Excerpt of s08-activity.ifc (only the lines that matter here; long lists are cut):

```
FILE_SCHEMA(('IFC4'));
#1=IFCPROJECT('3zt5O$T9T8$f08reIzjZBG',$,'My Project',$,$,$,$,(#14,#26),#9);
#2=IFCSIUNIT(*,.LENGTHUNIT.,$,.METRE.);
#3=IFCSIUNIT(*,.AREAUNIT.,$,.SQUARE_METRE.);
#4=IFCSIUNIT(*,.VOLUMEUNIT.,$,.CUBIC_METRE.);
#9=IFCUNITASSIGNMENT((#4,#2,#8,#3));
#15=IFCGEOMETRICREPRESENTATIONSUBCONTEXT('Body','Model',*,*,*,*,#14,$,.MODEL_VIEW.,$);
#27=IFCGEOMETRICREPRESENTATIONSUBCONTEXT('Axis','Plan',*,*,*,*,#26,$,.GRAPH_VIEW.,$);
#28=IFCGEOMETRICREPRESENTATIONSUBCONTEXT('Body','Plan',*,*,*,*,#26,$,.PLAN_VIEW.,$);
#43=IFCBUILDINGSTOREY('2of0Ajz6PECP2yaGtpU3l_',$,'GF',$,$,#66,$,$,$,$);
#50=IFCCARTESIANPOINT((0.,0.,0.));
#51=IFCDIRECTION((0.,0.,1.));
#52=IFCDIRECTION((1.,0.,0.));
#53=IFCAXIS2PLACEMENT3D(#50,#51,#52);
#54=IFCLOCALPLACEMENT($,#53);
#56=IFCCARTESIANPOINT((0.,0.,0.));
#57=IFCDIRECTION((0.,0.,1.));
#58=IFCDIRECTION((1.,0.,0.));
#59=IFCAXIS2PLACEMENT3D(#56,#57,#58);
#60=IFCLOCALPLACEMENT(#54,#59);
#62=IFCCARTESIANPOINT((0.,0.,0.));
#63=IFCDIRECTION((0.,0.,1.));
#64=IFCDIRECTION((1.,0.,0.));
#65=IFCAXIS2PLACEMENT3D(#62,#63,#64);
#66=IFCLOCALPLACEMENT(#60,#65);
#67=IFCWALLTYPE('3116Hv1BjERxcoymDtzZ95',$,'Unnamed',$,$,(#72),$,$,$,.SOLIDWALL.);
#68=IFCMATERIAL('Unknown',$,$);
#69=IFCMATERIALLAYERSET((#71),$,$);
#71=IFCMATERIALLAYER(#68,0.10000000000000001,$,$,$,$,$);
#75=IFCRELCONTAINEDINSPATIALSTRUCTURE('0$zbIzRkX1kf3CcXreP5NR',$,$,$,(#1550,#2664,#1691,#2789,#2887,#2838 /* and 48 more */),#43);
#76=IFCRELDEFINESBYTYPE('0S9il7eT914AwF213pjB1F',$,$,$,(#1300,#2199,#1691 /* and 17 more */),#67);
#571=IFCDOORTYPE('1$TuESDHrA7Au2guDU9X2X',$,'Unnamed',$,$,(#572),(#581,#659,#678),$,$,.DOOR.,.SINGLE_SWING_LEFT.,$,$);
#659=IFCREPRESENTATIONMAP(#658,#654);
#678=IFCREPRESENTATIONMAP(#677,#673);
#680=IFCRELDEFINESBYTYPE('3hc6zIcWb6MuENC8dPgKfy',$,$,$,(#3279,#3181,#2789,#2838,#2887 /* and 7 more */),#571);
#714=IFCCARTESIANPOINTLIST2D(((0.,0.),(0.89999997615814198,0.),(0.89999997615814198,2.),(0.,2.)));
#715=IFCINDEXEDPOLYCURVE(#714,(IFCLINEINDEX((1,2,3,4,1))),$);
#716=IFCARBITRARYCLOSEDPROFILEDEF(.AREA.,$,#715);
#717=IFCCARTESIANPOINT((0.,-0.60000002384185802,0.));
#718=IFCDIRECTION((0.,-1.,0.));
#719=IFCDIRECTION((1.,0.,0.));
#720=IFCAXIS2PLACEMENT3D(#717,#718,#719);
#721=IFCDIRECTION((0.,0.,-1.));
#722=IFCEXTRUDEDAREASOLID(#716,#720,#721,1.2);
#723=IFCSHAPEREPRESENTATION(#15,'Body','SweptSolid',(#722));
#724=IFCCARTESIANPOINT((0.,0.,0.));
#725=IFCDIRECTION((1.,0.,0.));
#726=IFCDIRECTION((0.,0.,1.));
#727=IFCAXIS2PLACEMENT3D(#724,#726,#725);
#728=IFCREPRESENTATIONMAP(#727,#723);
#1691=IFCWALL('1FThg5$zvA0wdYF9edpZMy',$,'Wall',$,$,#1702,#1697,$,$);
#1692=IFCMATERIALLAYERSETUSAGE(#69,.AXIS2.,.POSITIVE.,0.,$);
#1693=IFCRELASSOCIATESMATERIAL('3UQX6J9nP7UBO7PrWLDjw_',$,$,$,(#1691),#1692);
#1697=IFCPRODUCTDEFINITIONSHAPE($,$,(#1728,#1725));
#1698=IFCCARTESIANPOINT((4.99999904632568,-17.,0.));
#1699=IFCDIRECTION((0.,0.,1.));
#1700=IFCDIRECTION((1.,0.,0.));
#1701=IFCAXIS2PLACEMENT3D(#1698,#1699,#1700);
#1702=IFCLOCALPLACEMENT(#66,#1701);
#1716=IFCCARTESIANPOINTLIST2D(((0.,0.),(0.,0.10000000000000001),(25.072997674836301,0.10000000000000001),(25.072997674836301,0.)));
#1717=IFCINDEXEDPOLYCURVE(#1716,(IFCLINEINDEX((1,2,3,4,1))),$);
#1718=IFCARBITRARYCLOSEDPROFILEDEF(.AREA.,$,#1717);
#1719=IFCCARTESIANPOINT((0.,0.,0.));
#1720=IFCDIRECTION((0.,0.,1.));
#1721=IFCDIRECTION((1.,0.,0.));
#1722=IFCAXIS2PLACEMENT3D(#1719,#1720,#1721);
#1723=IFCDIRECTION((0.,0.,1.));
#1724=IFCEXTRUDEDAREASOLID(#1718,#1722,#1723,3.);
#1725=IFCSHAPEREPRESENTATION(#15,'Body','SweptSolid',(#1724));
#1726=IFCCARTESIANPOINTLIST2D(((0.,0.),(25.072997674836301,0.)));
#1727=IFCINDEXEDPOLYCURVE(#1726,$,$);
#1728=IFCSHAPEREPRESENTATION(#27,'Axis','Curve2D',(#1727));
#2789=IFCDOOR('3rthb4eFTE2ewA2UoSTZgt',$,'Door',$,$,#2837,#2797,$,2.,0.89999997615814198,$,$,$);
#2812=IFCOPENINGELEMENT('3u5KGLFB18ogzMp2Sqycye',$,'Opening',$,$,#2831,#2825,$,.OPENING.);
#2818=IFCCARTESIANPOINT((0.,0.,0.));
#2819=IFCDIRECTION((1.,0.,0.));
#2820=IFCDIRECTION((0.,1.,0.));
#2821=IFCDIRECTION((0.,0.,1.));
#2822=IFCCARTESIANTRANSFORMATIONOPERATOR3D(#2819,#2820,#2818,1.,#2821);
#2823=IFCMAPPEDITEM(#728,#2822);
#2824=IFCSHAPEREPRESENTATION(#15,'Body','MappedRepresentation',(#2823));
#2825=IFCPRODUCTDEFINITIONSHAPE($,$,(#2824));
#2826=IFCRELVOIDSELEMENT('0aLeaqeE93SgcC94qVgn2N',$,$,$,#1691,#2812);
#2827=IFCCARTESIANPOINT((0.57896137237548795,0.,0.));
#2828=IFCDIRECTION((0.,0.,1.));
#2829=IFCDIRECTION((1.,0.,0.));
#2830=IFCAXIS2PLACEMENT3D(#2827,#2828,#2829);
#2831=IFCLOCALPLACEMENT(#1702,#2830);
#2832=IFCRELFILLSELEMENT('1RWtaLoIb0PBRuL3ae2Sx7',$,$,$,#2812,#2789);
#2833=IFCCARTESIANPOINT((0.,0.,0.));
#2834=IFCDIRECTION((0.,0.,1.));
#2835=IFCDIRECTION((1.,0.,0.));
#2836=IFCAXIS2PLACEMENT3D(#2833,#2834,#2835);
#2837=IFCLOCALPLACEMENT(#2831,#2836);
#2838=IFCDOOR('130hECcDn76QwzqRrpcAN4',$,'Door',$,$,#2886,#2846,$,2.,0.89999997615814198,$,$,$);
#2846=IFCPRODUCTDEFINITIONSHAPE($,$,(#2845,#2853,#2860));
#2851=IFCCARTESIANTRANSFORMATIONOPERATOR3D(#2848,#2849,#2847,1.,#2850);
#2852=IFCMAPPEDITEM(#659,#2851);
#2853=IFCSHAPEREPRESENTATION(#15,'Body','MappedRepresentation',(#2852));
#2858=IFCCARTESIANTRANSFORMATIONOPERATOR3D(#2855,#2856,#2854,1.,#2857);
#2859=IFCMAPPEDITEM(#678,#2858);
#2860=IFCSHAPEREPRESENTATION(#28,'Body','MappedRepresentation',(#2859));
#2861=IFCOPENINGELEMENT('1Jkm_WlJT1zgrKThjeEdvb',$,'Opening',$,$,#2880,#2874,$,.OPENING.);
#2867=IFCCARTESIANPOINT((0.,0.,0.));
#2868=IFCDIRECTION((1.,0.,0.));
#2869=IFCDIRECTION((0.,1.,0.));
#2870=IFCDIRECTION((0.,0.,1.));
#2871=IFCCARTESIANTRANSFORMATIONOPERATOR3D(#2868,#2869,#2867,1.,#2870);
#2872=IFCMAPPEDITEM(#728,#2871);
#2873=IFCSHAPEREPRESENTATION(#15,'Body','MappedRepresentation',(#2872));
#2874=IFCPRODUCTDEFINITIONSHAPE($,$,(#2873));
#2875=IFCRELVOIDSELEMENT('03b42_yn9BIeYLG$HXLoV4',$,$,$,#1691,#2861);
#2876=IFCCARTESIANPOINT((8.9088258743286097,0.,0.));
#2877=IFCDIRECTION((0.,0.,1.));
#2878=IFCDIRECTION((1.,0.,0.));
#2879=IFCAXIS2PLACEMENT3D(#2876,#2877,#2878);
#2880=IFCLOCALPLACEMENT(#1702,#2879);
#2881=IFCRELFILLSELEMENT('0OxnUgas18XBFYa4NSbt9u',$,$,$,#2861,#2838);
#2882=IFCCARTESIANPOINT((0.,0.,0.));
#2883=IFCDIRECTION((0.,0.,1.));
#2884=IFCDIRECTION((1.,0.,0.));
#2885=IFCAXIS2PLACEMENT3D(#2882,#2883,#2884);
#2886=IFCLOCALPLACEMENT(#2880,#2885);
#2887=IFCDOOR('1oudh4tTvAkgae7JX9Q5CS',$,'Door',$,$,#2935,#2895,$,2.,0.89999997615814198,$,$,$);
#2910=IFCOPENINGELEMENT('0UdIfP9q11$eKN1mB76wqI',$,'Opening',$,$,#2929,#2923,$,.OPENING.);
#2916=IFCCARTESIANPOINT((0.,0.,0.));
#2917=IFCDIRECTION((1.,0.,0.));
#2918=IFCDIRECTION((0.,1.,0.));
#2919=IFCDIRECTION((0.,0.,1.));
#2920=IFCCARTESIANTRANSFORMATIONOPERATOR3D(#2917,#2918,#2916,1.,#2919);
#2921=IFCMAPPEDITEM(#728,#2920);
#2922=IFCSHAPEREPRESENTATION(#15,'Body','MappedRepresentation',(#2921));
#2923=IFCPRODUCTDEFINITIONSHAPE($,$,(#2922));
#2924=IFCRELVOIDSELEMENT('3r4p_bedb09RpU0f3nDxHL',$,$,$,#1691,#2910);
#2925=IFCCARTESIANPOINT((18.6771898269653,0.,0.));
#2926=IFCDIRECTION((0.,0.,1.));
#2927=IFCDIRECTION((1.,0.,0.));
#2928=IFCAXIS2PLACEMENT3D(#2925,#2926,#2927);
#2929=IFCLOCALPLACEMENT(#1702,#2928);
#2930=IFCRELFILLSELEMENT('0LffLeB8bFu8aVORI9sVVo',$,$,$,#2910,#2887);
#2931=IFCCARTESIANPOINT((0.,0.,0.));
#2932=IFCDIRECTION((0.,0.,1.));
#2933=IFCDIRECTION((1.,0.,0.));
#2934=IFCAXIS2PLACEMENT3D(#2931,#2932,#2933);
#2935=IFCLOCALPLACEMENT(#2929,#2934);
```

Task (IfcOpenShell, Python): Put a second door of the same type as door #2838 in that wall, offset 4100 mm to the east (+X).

```python
import ifcopenshell
import ifcopenshell.api.feature
import ifcopenshell.api.geometry
import ifcopenshell.api.root
import ifcopenshell.geom
import ifcopenshell.util.element
import ifcopenshell.util.placement
import ifcopenshell.util.shape

model = ifcopenshell.open("s08-activity.ifc")
settings = ifcopenshell.geom.settings()


def volume(element):
    """Net volume in cubic metres, openings subtracted."""
    shape = ifcopenshell.geom.create_shape(settings, element)
    return ifcopenshell.util.shape.get_volume(shape.geometry)


door = model.by_id(2838)
opening = door.FillsVoids[0].RelatingOpeningElement
wall = opening.VoidsElements[0].RelatingBuildingElement
before = volume(wall)
shift = ifcopenshell.util.placement.get_local_placement(wall.ObjectPlacement)[:3, 0] * 4.1

# copy_class copies the void relationship, type, container and properties, but no geometry.
new_opening = ifcopenshell.api.root.copy_class(model, product=opening)
new_opening.Representation = ifcopenshell.util.element.copy_deep(
    model, opening.Representation, exclude=["IfcGeometricRepresentationContext", "IfcRepresentationMap"]
)
new_door = ifcopenshell.api.root.copy_class(model, product=door)
new_door.Representation = ifcopenshell.util.element.copy_deep(
    model, door.Representation, exclude=["IfcGeometricRepresentationContext", "IfcRepresentationMap"]
)
ifcopenshell.api.feature.add_filling(model, opening=new_opening, element=new_door)

for old, new in ((opening, new_opening), (door, new_door)):
    matrix = ifcopenshell.util.placement.get_local_placement(old.ObjectPlacement)
    matrix[:3, 3] += shift
    ifcopenshell.api.geometry.edit_object_placement(model, product=new, matrix=matrix, is_si=False)

after = volume(wall)

print(f"wall volume {before:.3f} -> {after:.3f} m3")

model.write("s08-activity_v2.ifc")
```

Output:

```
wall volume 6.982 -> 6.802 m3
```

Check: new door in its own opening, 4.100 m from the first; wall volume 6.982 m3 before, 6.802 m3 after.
